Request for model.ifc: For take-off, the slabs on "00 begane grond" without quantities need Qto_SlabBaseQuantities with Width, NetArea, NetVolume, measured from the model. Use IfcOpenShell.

First a look at what the model holds.

```python
import ifcopenshell
import ifcopenshell.util.element
import ifcopenshell.util.unit

model = ifcopenshell.open("model.ifc")
print(model.schema)
for unit_type in ("LENGTHUNIT", "AREAUNIT", "VOLUMEUNIT"):
    print(unit_type, ifcopenshell.util.unit.calculate_unit_scale(model, unit_type))
storey = next(s for s in model.by_type("IfcBuildingStorey") if s.Name == "00 begane grond")
slabs = [e for e in ifcopenshell.util.element.get_decomposition(storey) if e.is_a("IfcSlab")]
for e in sorted(slabs, key=lambda e: e.id()):
    print(e.id(), e.is_a(), e.Name, list(ifcopenshell.util.element.get_psets(e, qtos_only=True)), sep=" | ")
```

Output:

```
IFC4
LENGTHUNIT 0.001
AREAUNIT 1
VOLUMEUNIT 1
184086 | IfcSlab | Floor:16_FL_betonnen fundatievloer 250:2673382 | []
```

```python
import ifcopenshell
import ifcopenshell.api.pset
import ifcopenshell.geom
import ifcopenshell.util.element
import ifcopenshell.util.shape
import ifcopenshell.util.unit

model = ifcopenshell.open("model.ifc")
unit_scale = ifcopenshell.util.unit.calculate_unit_scale(model)
area_scale = ifcopenshell.util.unit.calculate_unit_scale(model, "AREAUNIT")
volume_scale = ifcopenshell.util.unit.calculate_unit_scale(model, "VOLUMEUNIT")
settings = ifcopenshell.geom.settings()

storey = next(s for s in model.by_type("IfcBuildingStorey") if s.Name == "00 begane grond")
slabs = [e for e in ifcopenshell.util.element.get_decomposition(storey) if e.is_a("IfcSlab")]

for e in sorted(slabs, key=lambda e: e.id()):
    if ifcopenshell.util.element.get_psets(e, qtos_only=True, should_inherit=False):
        continue
    # Geometry comes back in metres, in the element's own axes.
    shape = ifcopenshell.geom.create_shape(settings, e)
    values = {
        "Width": ifcopenshell.util.shape.get_z(shape.geometry) / unit_scale,
        "NetArea": ifcopenshell.util.shape.get_footprint_area(shape.geometry) / area_scale,
        "NetVolume": ifcopenshell.util.shape.get_volume(shape.geometry) / volume_scale,
    }
    qto = ifcopenshell.api.pset.add_qto(model, product=e, name="Qto_SlabBaseQuantities")
    ifcopenshell.api.pset.edit_qto(model, qto=qto, properties=values)
    print(e.id(), {k: round(v, 3) for k, v in values.items()})

model.write("model_rev.ifc")
```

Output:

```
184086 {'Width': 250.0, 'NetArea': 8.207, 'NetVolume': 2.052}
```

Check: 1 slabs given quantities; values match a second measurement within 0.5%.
